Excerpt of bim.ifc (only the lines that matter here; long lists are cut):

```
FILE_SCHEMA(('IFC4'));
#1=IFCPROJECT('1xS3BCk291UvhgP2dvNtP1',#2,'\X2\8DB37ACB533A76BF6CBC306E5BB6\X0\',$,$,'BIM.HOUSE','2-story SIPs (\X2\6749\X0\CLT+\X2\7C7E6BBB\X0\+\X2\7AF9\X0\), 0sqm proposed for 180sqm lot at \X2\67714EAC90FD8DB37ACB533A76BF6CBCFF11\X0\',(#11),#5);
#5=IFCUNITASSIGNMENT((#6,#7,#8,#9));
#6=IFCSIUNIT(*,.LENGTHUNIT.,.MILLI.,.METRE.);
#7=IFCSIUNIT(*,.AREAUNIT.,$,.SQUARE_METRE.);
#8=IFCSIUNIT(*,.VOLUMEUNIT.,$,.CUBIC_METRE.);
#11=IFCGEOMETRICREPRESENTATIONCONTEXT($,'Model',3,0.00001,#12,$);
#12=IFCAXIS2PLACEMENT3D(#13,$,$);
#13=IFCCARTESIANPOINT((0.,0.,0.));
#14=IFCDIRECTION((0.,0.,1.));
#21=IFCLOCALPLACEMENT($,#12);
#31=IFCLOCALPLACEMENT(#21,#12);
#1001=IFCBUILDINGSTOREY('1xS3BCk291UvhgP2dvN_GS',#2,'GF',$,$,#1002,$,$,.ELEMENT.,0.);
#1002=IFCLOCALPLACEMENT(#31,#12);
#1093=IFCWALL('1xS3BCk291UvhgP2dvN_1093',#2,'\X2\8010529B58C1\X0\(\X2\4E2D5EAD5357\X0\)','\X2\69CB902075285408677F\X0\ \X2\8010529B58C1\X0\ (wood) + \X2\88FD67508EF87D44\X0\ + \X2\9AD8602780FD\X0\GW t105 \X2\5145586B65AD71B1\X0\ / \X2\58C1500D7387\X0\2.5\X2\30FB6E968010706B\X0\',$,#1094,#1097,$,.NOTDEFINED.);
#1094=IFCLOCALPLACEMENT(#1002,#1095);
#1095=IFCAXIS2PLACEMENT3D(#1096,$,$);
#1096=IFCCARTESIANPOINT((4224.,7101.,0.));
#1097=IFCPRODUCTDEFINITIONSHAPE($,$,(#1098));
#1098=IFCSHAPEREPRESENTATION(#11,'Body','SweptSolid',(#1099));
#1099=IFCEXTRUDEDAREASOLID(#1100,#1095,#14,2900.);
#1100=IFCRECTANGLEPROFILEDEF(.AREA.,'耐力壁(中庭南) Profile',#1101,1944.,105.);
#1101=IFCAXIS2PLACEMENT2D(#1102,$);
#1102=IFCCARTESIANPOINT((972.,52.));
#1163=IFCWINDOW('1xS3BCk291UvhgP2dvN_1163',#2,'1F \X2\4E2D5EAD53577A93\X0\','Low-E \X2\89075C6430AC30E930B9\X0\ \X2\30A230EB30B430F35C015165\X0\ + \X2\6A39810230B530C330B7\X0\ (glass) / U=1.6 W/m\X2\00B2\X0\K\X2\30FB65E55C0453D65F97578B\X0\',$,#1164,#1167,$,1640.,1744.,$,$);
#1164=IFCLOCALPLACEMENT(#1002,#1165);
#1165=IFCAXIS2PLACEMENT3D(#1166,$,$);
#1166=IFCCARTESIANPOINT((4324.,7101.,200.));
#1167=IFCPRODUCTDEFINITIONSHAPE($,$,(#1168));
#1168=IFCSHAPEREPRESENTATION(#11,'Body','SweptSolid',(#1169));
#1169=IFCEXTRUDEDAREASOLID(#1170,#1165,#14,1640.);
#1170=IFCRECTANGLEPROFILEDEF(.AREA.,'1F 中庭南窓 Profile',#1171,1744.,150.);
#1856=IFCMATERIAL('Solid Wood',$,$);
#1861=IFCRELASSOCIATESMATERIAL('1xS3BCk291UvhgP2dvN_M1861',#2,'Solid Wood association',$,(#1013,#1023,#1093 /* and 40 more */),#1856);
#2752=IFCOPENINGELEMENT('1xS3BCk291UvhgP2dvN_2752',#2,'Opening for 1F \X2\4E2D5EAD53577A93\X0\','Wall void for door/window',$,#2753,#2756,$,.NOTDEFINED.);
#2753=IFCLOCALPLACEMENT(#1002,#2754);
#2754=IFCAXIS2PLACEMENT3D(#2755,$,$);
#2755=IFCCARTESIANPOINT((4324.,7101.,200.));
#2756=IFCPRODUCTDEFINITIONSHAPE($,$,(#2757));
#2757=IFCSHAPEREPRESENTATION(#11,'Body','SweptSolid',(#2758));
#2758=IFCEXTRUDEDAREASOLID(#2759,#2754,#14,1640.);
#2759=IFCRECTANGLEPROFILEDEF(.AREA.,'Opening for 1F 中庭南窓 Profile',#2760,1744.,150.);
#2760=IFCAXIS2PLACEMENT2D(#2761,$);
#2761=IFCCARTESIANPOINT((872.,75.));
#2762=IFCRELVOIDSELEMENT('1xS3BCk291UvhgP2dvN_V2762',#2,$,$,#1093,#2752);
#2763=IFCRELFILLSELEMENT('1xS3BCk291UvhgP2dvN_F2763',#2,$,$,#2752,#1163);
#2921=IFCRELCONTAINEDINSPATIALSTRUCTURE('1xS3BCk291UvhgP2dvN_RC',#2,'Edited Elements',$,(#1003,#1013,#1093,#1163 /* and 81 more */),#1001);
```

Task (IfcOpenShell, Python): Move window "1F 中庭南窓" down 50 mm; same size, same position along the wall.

```python
import numpy as np
import ifcopenshell
import ifcopenshell.api.geometry
import ifcopenshell.util.placement
import ifcopenshell.util.unit

model = ifcopenshell.open("bim.ifc")
unit_scale = ifcopenshell.util.unit.calculate_unit_scale(model)

window = model.by_id(1163)
opening = window.FillsVoids[0].RelatingOpeningElement
dz = -50.0

shift = np.array([0.0, 0.0, dz])
# The window is not placed relative to its opening, so move both.
for product in (opening, window):
    matrix = ifcopenshell.util.placement.get_local_placement(product.ObjectPlacement)
    matrix[:3, 3] += shift
    ifcopenshell.api.geometry.edit_object_placement(model, product=product, matrix=matrix, is_si=False)

print(f"moved by {dz * unit_scale:+.3f} m")

model.write("bim_v2.ifc")
```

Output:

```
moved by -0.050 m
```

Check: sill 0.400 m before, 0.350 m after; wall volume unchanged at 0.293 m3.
